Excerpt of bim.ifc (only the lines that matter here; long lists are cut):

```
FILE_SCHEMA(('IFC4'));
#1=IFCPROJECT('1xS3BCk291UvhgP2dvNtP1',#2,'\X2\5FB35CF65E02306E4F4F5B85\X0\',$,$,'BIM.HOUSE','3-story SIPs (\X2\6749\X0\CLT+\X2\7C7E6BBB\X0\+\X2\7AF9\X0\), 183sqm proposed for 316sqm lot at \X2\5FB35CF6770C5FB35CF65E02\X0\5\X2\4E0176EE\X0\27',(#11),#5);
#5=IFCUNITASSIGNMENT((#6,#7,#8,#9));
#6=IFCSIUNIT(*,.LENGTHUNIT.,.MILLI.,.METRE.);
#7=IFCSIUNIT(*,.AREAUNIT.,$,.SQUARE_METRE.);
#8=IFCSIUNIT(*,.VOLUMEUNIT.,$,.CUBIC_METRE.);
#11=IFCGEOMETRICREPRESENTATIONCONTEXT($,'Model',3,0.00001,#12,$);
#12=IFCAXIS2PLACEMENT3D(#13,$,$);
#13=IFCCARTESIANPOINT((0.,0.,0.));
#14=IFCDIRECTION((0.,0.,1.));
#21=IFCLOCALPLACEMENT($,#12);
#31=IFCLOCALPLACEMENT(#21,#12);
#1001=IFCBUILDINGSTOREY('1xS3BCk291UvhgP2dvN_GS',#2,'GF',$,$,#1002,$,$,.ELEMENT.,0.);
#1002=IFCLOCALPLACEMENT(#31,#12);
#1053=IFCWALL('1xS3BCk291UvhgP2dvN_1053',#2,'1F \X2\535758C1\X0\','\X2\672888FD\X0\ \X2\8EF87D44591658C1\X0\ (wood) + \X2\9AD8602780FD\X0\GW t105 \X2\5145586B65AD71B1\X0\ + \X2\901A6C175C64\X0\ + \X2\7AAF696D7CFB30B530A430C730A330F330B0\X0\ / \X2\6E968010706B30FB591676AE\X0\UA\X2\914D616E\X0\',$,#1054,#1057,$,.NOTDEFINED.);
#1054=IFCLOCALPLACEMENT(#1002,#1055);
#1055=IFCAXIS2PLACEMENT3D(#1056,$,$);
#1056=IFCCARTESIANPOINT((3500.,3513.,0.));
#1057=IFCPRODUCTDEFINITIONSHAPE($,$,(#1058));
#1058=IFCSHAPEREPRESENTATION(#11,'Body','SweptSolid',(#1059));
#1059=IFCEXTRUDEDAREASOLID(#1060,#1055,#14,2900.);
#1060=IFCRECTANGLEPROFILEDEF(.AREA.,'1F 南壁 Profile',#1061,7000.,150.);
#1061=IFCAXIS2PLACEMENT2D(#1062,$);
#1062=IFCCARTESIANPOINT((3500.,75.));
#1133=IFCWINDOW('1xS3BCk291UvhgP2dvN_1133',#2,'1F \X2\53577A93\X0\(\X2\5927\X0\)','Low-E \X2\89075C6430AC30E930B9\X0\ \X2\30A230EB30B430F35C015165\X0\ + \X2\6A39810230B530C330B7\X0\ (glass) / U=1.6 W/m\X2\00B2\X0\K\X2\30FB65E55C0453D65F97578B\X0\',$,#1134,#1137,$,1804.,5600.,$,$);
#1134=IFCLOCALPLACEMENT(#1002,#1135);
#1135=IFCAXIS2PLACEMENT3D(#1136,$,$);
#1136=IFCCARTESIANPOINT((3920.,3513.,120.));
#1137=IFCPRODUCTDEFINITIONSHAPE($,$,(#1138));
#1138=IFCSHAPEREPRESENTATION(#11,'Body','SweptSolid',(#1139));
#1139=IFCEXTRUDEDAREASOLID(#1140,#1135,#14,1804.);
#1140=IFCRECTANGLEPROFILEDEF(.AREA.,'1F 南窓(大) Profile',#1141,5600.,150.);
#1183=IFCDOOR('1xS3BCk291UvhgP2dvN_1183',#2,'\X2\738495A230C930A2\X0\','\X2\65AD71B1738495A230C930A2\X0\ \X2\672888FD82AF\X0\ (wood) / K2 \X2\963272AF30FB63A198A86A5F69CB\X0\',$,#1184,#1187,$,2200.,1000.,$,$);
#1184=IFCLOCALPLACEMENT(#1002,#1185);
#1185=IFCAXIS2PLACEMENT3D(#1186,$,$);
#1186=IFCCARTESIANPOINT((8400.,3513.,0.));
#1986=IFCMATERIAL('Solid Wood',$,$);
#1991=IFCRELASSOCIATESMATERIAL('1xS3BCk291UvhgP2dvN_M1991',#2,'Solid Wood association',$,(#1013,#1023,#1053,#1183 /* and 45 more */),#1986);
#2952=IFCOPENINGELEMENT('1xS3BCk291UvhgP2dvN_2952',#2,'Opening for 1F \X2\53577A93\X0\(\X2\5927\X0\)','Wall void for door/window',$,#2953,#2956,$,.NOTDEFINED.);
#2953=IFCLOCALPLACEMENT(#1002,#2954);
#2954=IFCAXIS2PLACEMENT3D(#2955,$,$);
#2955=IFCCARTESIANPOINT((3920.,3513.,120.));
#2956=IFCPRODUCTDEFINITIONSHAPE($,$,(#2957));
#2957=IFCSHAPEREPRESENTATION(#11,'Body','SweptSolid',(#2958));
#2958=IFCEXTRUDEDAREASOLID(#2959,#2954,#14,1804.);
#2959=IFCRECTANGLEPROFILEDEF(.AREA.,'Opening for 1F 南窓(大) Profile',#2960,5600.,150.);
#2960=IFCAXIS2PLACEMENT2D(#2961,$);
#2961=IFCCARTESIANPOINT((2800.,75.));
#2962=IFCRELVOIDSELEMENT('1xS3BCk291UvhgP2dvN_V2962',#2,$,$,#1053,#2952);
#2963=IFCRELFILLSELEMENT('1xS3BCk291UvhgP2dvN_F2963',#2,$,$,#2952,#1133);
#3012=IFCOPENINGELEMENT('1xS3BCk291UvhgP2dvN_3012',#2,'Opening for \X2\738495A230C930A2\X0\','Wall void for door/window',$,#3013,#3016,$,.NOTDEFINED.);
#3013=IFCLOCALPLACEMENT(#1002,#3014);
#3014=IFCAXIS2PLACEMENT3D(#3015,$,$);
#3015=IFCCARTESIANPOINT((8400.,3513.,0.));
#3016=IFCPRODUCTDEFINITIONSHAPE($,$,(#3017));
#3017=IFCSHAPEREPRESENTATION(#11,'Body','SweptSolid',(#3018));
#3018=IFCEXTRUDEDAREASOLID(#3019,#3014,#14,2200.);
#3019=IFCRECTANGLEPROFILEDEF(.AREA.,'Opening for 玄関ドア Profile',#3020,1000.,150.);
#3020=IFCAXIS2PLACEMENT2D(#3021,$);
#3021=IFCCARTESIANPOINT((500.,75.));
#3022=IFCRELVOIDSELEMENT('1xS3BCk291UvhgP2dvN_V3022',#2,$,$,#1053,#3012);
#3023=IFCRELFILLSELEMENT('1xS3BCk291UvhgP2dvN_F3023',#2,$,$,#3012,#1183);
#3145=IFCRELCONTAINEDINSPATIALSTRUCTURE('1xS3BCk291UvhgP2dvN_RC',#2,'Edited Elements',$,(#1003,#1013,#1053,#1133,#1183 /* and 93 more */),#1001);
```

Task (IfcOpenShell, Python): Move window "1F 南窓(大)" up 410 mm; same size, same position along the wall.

```python
import numpy as np
import ifcopenshell
import ifcopenshell.api.geometry
import ifcopenshell.util.placement
import ifcopenshell.util.unit

model = ifcopenshell.open("bim.ifc")
unit_scale = ifcopenshell.util.unit.calculate_unit_scale(model)

window = model.by_id(1133)
opening = window.FillsVoids[0].RelatingOpeningElement
dz = 0.41 / unit_scale

shift = np.array([0.0, 0.0, dz])
# The window is not placed relative to its opening, so move both.
for product in (opening, window):
    matrix = ifcopenshell.util.placement.get_local_placement(product.ObjectPlacement)
    matrix[:3, 3] += shift
    ifcopenshell.api.geometry.edit_object_placement(model, product=product, matrix=matrix, is_si=False)

print(f"moved by {dz * unit_scale:+.3f} m")

model.write("bim_updated.ifc")
```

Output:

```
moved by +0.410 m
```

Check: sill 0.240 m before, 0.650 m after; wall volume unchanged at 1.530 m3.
